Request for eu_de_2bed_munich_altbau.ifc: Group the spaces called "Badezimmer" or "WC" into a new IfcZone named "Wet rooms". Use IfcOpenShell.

First a look at what the model holds.

```python
import ifcopenshell

model = ifcopenshell.open("eu_de_2bed_munich_altbau.ifc")
print(model.schema)
seen = {}
for space in model.by_type("IfcSpace"):
    seen[space.LongName] = seen.get(space.LongName, 0) + 1
for name, count in sorted(seen.items(), key=str):
    print(count, "x", name)
print("zones:", [z.Name for z in model.by_type("IfcZone")][:20])
```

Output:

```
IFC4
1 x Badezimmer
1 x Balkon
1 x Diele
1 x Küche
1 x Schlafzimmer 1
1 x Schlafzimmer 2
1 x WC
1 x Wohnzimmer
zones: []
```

```python
import ifcopenshell
import ifcopenshell.api.group
import ifcopenshell.api.root

model = ifcopenshell.open("eu_de_2bed_munich_altbau.ifc")

names = {"Badezimmer", "WC"}
spaces = [s for s in model.by_type("IfcSpace") if s.LongName in names]

zone = ifcopenshell.api.root.create_entity(model, ifc_class="IfcZone", name="Wet rooms")
ifcopenshell.api.group.assign_group(model, products=spaces, group=zone)
print(len(spaces), "spaces in", zone.Name)

model.write("eu_de_2bed_munich_altbau_v2.ifc")
```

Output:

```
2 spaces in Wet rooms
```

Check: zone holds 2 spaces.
